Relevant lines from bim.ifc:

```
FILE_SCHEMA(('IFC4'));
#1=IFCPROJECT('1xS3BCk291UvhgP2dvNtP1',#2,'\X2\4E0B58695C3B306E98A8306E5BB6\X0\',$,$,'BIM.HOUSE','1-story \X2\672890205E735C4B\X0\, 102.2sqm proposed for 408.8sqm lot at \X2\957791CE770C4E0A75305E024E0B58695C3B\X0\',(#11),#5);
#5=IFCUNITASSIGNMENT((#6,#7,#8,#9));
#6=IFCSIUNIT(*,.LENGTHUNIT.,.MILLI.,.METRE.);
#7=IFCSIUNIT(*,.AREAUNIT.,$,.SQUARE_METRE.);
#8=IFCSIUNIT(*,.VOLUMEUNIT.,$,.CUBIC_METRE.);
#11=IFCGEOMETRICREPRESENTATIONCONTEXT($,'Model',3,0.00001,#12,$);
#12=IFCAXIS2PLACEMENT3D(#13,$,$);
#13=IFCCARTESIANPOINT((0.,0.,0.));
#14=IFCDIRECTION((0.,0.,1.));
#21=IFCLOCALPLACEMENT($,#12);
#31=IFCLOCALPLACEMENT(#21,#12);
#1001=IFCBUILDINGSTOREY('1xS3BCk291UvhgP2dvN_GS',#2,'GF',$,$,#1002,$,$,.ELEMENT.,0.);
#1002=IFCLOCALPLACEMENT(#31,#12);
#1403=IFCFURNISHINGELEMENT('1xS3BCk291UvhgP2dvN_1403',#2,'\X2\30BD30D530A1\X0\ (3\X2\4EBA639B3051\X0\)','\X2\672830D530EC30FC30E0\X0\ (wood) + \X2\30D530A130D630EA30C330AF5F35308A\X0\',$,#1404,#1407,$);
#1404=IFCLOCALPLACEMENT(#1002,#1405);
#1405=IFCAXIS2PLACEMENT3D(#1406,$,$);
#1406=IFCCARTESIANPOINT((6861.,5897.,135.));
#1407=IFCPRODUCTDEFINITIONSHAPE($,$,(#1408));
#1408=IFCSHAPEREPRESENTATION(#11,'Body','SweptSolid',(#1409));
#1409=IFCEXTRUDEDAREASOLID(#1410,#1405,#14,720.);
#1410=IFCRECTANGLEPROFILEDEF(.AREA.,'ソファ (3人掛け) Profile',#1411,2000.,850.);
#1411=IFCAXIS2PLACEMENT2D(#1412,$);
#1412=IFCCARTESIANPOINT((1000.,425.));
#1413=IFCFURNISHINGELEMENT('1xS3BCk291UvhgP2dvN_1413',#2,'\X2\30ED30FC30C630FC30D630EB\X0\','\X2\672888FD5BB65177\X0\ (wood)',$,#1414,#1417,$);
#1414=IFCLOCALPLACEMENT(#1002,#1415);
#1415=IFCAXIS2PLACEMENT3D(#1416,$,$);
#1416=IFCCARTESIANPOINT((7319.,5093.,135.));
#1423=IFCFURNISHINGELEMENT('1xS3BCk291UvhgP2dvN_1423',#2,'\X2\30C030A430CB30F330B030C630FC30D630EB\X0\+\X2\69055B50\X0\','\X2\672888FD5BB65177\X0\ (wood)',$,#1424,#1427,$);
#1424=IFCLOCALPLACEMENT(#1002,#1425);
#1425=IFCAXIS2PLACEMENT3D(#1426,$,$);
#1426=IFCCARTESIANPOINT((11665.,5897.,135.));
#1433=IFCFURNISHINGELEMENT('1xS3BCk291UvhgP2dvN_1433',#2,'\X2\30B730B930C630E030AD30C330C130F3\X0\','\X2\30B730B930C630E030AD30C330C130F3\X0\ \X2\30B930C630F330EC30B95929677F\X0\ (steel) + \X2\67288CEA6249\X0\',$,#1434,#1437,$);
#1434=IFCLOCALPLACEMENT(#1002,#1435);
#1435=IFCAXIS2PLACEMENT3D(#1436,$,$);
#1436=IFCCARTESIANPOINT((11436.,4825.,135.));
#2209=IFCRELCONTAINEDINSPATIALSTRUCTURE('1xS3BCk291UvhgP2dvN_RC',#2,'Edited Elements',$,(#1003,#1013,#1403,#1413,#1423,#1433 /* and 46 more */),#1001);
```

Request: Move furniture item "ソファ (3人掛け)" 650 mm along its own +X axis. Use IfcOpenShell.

```python
import ifcopenshell
import ifcopenshell.api.geometry
import ifcopenshell.util.placement
import ifcopenshell.util.unit

model = ifcopenshell.open("bim.ifc")
unit_scale = ifcopenshell.util.unit.calculate_unit_scale(model)

item = model.by_guid("1xS3BCk291UvhgP2dvN_1403")
matrix = ifcopenshell.util.placement.get_local_placement(item.ObjectPlacement)
matrix[:3, 3] += matrix[:3, 0] * 0.65 / unit_scale
ifcopenshell.api.geometry.edit_object_placement(model, product=item, matrix=matrix, is_si=False)

print(ifcopenshell.util.placement.get_local_placement(item.ObjectPlacement).round(3) + 0.0)

model.write("bim-out.ifc")
```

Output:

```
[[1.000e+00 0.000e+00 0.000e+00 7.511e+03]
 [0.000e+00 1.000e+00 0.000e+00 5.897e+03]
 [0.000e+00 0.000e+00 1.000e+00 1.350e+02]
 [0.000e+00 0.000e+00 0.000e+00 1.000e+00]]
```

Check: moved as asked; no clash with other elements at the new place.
